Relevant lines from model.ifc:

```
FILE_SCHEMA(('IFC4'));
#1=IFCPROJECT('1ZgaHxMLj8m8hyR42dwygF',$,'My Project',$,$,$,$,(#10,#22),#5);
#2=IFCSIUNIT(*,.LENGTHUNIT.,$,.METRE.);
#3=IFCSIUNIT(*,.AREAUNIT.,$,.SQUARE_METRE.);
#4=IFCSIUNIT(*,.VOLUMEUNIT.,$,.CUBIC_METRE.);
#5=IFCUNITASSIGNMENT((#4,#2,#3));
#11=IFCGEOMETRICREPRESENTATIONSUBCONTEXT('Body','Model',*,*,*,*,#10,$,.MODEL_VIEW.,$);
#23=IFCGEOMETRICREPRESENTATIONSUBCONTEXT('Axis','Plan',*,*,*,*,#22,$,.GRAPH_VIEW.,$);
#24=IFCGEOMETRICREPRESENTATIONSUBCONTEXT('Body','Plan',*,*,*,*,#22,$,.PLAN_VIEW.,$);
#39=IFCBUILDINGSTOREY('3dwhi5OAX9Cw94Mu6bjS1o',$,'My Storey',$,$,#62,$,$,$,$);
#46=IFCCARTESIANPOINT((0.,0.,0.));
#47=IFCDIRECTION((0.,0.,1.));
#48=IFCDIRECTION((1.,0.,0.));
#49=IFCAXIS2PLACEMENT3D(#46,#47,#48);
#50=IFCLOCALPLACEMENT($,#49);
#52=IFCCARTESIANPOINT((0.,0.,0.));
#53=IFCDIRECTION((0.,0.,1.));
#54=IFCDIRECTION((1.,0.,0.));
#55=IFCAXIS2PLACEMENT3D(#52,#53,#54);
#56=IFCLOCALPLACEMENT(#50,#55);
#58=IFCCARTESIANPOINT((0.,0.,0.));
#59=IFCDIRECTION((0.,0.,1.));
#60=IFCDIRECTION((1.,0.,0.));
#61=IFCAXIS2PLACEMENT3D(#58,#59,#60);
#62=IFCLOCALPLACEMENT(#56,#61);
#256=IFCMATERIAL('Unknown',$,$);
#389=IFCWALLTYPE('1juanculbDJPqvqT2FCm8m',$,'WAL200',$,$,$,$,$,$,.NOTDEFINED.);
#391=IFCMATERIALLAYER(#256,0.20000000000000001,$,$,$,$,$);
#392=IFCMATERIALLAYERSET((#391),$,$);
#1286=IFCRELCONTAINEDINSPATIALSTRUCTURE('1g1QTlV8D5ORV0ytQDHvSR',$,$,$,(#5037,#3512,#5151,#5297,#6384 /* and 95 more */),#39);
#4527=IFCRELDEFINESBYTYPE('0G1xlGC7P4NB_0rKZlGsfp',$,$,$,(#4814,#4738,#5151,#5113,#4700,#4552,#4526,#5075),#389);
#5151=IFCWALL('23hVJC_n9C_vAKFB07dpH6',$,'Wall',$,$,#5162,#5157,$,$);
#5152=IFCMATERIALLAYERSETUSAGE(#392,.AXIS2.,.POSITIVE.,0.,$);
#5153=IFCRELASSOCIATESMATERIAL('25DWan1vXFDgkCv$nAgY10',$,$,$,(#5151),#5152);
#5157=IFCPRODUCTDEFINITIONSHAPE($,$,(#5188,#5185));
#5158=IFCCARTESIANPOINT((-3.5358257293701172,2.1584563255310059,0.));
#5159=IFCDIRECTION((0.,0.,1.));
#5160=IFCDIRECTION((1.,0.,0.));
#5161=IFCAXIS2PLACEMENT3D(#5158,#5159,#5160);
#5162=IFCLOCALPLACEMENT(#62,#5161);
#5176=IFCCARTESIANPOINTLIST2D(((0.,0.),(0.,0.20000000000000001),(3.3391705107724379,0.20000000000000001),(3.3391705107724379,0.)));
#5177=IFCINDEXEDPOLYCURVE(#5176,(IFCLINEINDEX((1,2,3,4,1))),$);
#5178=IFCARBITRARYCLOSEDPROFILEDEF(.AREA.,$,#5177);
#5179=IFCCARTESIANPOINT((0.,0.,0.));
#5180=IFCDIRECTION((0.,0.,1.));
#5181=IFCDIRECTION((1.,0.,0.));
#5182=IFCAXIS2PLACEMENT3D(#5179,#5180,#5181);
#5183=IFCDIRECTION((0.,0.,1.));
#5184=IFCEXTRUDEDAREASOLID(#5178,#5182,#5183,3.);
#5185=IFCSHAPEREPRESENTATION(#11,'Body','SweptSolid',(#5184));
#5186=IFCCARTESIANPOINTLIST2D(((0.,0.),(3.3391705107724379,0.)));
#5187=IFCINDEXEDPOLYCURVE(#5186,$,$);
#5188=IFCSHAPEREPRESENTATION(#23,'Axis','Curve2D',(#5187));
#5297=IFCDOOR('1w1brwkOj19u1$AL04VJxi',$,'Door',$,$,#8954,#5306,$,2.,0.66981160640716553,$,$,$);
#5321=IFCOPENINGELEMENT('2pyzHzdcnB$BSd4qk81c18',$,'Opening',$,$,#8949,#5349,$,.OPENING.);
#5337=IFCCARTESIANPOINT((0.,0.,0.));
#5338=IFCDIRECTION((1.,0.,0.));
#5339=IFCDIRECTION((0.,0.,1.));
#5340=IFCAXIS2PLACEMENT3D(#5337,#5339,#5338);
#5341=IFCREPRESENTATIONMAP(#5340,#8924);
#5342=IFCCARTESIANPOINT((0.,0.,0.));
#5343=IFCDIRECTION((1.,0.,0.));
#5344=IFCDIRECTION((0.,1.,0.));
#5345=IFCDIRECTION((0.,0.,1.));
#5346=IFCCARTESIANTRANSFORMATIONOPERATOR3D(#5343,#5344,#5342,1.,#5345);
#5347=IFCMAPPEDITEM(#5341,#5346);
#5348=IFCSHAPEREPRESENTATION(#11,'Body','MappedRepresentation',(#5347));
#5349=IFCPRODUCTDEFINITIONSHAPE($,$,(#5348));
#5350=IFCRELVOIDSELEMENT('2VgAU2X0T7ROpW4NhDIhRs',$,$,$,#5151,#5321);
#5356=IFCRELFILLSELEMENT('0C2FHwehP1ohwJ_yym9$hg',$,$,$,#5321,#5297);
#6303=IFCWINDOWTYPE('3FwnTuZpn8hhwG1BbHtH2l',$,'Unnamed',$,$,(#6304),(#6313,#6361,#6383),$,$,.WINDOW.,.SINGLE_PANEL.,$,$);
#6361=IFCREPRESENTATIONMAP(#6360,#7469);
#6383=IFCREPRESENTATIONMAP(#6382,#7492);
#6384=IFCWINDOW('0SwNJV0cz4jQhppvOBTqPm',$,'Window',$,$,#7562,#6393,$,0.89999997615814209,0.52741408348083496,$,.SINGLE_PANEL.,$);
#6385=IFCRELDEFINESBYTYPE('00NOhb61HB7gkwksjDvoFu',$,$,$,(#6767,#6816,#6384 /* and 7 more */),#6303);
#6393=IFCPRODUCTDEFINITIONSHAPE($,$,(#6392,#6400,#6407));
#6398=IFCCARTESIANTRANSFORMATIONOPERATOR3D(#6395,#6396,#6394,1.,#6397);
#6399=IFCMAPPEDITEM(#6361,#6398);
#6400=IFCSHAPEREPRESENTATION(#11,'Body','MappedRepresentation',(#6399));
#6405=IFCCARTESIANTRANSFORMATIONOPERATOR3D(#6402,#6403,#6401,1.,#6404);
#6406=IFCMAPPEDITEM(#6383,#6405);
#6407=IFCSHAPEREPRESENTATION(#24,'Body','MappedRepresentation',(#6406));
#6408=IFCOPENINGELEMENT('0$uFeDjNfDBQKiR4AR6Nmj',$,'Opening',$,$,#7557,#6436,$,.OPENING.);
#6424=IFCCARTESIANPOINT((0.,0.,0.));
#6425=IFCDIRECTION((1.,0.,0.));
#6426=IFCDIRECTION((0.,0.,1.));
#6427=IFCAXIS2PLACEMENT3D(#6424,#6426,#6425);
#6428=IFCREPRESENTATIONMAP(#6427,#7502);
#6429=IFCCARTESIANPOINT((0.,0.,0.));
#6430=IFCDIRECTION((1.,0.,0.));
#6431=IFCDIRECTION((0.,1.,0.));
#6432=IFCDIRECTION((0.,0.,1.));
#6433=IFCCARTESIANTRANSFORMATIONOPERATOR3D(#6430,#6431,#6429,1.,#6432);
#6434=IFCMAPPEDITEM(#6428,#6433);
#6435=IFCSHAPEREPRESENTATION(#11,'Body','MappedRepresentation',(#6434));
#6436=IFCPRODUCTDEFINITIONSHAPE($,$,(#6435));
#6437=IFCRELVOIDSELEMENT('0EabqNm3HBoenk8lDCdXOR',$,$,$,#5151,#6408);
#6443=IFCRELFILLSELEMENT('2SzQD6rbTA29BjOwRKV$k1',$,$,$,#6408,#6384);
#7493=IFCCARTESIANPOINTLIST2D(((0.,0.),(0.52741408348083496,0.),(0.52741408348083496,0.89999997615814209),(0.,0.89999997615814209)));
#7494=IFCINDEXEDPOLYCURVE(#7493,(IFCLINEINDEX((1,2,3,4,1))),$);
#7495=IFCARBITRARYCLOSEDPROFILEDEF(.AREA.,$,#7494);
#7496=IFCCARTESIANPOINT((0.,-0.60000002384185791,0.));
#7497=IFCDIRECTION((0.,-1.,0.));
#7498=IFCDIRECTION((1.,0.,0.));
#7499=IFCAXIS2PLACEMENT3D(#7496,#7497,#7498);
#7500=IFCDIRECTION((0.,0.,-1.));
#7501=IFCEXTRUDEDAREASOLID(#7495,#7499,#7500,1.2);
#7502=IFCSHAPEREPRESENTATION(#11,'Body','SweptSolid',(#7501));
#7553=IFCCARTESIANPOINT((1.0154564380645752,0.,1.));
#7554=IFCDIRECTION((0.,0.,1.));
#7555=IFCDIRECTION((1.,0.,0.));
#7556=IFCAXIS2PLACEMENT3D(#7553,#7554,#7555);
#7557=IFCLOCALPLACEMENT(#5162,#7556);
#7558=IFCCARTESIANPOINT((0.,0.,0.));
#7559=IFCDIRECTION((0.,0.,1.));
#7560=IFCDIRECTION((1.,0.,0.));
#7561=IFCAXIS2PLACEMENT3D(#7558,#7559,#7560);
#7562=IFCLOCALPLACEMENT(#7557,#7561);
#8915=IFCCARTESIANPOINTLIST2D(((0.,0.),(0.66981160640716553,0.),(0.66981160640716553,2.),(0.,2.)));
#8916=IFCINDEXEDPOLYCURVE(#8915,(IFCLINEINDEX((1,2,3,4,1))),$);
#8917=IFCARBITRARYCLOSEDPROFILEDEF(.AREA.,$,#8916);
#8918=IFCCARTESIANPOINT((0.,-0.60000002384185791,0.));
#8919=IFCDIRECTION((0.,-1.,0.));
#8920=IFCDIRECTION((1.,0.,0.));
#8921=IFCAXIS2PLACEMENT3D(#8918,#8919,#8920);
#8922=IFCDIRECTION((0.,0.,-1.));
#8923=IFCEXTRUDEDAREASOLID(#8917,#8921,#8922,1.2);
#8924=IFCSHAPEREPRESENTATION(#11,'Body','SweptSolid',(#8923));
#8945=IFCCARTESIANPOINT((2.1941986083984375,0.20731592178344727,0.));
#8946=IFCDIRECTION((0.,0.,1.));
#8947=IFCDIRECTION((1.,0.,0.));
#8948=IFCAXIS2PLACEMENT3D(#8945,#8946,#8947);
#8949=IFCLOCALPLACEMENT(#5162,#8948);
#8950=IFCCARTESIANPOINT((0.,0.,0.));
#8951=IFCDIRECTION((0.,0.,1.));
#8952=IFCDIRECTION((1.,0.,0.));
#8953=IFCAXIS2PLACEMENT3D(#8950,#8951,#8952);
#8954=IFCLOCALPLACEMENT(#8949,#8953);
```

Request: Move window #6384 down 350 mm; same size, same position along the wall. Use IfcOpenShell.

```python
import numpy as np
import ifcopenshell
import ifcopenshell.api.geometry
import ifcopenshell.util.placement
import ifcopenshell.util.unit

model = ifcopenshell.open("model.ifc")
unit_scale = ifcopenshell.util.unit.calculate_unit_scale(model)

window = model.by_id(6384)
opening = window.FillsVoids[0].RelatingOpeningElement
dz = -0.35

shift = np.array([0.0, 0.0, dz])
# The window is placed relative to its opening, so it follows when the opening moves.
matrix = ifcopenshell.util.placement.get_local_placement(opening.ObjectPlacement)
matrix[:3, 3] += shift
ifcopenshell.api.geometry.edit_object_placement(
    model, product=opening, matrix=matrix, is_si=False, should_transform_children=True
)

print(f"moved by {dz * unit_scale:+.3f} m")

model.write("model_edited.ifc")
```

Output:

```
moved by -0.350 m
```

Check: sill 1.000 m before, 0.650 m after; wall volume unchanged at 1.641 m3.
